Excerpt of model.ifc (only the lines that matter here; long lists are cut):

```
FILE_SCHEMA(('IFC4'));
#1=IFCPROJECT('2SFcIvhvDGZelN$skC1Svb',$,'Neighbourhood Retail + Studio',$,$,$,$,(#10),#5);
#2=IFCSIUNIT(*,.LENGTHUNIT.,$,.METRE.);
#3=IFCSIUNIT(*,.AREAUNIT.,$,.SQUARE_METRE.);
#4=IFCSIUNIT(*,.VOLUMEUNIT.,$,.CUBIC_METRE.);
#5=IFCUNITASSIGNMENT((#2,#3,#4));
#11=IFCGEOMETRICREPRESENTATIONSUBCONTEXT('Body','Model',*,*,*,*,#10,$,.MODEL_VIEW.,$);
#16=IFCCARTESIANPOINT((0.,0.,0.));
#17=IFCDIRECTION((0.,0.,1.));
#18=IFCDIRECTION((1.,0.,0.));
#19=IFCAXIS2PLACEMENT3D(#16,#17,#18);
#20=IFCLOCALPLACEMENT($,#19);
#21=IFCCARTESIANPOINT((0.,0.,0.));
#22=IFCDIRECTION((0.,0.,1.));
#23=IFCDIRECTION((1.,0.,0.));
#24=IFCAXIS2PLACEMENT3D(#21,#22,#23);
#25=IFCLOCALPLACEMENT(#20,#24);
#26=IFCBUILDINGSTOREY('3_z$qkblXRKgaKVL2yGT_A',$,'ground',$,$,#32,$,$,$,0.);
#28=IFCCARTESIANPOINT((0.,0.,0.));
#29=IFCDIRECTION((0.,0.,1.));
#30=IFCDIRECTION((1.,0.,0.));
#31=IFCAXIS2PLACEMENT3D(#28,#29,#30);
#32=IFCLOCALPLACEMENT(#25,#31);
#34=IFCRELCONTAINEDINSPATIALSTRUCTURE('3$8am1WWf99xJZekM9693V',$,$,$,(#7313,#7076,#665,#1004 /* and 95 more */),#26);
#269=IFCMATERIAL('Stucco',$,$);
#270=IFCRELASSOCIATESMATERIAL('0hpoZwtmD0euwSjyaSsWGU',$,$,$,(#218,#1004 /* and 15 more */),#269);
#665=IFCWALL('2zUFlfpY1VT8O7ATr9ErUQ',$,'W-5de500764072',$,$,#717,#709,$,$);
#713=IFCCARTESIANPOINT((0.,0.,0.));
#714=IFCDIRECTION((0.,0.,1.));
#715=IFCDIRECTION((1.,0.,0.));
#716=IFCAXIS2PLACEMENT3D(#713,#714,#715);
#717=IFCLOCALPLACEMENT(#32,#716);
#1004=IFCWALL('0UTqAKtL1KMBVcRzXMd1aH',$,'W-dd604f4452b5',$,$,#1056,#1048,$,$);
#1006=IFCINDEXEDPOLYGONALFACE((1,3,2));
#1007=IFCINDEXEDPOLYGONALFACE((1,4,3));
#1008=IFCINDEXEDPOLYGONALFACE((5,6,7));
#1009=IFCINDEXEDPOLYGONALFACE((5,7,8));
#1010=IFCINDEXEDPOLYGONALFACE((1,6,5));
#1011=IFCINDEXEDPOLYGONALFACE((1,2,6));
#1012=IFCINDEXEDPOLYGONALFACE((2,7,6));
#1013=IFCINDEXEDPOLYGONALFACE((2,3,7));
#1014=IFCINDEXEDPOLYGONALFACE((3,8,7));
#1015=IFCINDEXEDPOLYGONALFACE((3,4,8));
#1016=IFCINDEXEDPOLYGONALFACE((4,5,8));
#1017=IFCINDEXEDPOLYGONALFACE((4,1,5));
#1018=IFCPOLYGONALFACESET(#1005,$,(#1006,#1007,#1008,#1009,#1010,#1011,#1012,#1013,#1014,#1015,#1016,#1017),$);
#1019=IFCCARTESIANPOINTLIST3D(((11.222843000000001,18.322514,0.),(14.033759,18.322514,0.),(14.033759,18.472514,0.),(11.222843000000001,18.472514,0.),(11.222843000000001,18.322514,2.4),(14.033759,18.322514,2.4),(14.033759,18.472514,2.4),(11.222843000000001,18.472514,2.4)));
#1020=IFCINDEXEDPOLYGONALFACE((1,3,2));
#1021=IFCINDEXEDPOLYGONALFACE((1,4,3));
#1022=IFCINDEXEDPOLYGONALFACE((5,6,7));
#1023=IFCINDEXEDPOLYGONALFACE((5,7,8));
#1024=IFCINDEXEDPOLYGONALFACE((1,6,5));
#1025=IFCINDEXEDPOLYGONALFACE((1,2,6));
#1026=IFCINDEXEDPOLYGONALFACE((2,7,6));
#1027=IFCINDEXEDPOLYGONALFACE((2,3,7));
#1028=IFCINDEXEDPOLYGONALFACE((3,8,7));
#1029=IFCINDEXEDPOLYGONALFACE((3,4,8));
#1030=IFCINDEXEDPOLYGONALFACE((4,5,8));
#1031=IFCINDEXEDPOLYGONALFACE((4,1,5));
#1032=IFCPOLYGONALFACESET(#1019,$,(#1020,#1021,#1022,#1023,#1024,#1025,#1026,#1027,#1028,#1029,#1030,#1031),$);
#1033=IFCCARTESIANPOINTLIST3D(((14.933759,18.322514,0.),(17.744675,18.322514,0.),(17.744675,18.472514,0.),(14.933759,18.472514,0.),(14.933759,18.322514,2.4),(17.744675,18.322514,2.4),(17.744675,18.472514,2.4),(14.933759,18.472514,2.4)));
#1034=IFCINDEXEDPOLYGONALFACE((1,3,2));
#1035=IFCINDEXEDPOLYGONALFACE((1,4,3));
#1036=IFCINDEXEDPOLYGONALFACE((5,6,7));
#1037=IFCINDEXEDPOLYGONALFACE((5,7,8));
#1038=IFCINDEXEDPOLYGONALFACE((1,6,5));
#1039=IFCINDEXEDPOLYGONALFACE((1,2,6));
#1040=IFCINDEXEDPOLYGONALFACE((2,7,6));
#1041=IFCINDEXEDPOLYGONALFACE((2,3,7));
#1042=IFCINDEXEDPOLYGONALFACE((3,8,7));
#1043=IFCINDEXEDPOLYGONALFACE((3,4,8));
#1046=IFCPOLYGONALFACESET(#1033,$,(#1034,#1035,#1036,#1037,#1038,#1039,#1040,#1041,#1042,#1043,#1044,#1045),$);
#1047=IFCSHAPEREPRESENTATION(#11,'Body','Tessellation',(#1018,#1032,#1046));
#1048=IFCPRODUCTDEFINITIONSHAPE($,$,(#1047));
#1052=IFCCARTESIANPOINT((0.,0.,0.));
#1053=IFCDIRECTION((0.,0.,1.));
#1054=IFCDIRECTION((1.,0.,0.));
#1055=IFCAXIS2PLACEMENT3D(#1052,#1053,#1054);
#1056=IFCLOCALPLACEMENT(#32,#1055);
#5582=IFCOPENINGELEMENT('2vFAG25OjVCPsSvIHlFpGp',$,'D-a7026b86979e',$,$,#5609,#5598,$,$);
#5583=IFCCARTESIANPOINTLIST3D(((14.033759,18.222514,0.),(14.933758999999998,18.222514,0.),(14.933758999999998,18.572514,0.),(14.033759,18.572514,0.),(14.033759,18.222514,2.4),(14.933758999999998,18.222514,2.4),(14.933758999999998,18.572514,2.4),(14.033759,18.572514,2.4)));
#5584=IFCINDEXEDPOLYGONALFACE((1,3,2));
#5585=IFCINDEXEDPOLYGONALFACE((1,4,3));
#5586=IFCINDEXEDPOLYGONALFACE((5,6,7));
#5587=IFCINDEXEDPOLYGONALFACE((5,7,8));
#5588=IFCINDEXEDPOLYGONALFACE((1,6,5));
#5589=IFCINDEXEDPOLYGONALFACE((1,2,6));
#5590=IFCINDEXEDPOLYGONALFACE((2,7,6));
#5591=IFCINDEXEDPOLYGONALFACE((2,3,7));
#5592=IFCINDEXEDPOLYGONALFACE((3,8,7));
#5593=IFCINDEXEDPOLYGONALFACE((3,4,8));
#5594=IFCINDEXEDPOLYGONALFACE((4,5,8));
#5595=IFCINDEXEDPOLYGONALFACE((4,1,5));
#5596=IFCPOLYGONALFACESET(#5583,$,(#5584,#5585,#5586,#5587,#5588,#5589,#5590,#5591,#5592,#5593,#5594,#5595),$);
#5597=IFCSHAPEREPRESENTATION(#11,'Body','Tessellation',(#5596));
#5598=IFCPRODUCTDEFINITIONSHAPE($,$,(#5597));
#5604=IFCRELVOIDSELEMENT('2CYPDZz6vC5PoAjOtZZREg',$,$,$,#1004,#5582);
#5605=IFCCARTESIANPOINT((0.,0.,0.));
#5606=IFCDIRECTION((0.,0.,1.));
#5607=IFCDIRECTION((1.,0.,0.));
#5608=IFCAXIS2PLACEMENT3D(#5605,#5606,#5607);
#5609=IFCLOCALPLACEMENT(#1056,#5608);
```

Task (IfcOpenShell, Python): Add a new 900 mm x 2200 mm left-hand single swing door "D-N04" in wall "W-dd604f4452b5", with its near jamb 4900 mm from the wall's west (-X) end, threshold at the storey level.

```python
import numpy as np
import ifcopenshell
import ifcopenshell.api.feature
import ifcopenshell.api.geometry
import ifcopenshell.api.root
import ifcopenshell.api.spatial
import ifcopenshell.geom
import ifcopenshell.util.element
import ifcopenshell.util.placement
import ifcopenshell.util.representation
import ifcopenshell.util.shape
import ifcopenshell.util.unit

model = ifcopenshell.open("model.ifc")
unit_scale = ifcopenshell.util.unit.calculate_unit_scale(model)
settings = ifcopenshell.geom.settings()


def volume(element):
    """Net volume in cubic metres, openings subtracted."""
    shape = ifcopenshell.geom.create_shape(settings, element)
    return ifcopenshell.util.shape.get_volume(shape.geometry)


wall = model.by_guid("0UTqAKtL1KMBVcRzXMd1aH")
storey = ifcopenshell.util.element.get_container(wall, ifc_class="IfcBuildingStorey")
context = ifcopenshell.util.representation.get_context(model, "Model", "Body", "MODEL_VIEW")
before = volume(wall)

width, height, from_end, sill = 0.9, 2.2, 4.9, 0.0  # metres

# The wall runs along its own X axis, and the end named is its -X end.
wall_shape = ifcopenshell.geom.create_shape(settings, wall)
x, y, z = ifcopenshell.util.shape.get_vertices(wall_shape.geometry).T
start = x.min() + from_end
face, thickness = float(y.min()), float(y.max() - y.min())
wall_matrix = ifcopenshell.util.placement.get_local_placement(wall.ObjectPlacement)
level = ifcopenshell.util.placement.get_local_placement(storey.ObjectPlacement)[2, 3]


def in_wall(x, y):
    """Placement at x, y metres in the wall's axes, at sill height."""
    matrix = wall_matrix.copy()
    matrix[:, 3] = wall_matrix @ np.array([x / unit_scale, y / unit_scale, 0.0, 1.0])
    matrix[2, 3] = level + sill / unit_scale
    return matrix


# Opening: a box that overshoots both wall faces by 50 mm.
opening = ifcopenshell.api.root.create_entity(model, ifc_class="IfcOpeningElement", predefined_type="OPENING")
box = ifcopenshell.api.geometry.add_wall_representation(
    model, context=context, length=width, height=height, thickness=thickness + 0.1
)
ifcopenshell.api.geometry.assign_representation(model, product=opening, representation=box)
ifcopenshell.api.geometry.edit_object_placement(model, product=opening, matrix=in_wall(start, face - 0.05), is_si=False)
ifcopenshell.api.feature.add_feature(model, feature=opening, element=wall)

door = ifcopenshell.api.root.create_entity(model, ifc_class="IfcDoor", name="D-N04", predefined_type="DOOR")
door.OverallWidth, door.OverallHeight = width / unit_scale, height / unit_scale
door.OperationType = "SINGLE_SWING_LEFT"
body = ifcopenshell.api.geometry.add_door_representation(
    model,
    context=context,
    overall_width=door.OverallWidth,
    overall_height=door.OverallHeight,
    operation_type="SINGLE_SWING_LEFT",
    lining_properties={"LiningDepth": thickness / unit_scale, "ThresholdDepth": thickness / unit_scale},
)
ifcopenshell.api.geometry.assign_representation(model, product=door, representation=body)
ifcopenshell.api.spatial.assign_container(model, products=[door], relating_structure=storey)
ifcopenshell.api.feature.add_filling(model, opening=opening, element=door)

# The lining spans the wall, so the door starts at the wall face.
ifcopenshell.api.geometry.edit_object_placement(model, product=door, matrix=in_wall(start, face), is_si=False)

after = volume(wall)

print(f"wall volume {before:.3f} -> {after:.3f} m3")

model.write("model_updated.ifc")
```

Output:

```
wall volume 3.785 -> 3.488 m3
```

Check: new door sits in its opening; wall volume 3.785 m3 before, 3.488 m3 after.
